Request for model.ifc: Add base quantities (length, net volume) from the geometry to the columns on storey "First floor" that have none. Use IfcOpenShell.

First a look at what the model holds.

```python
import ifcopenshell
import ifcopenshell.util.element
import ifcopenshell.util.unit

model = ifcopenshell.open("model.ifc")
print(model.schema)
for unit_type in ("LENGTHUNIT", "AREAUNIT", "VOLUMEUNIT"):
    print(unit_type, ifcopenshell.util.unit.calculate_unit_scale(model, unit_type))
storey = next(s for s in model.by_type("IfcBuildingStorey") if s.Name == "First floor")
columns = [e for e in ifcopenshell.util.element.get_decomposition(storey) if e.is_a("IfcColumn")]
for e in sorted(columns, key=lambda e: e.id()):
    print(e.id(), e.is_a(), e.Name, list(ifcopenshell.util.element.get_psets(e, qtos_only=True)), sep=" | ")
```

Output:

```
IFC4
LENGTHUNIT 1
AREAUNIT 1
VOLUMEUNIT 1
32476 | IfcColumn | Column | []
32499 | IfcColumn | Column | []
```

```python
import ifcopenshell
import ifcopenshell.api.pset
import ifcopenshell.geom
import ifcopenshell.util.element
import ifcopenshell.util.shape
import ifcopenshell.util.unit

model = ifcopenshell.open("model.ifc")
unit_scale = ifcopenshell.util.unit.calculate_unit_scale(model)
volume_scale = ifcopenshell.util.unit.calculate_unit_scale(model, "VOLUMEUNIT")
settings = ifcopenshell.geom.settings()

storey = next(s for s in model.by_type("IfcBuildingStorey") if s.Name == "First floor")
columns = [e for e in ifcopenshell.util.element.get_decomposition(storey) if e.is_a("IfcColumn")]

for e in sorted(columns, key=lambda e: e.id()):
    if ifcopenshell.util.element.get_psets(e, qtos_only=True, should_inherit=False):
        continue
    # Geometry comes back in metres, in the element's own axes.
    shape = ifcopenshell.geom.create_shape(settings, e)
    values = {
        "Length": ifcopenshell.util.shape.get_z(shape.geometry) / unit_scale,
        "NetVolume": ifcopenshell.util.shape.get_volume(shape.geometry) / volume_scale,
    }
    qto = ifcopenshell.api.pset.add_qto(model, product=e, name="Qto_ColumnBaseQuantities")
    ifcopenshell.api.pset.edit_qto(model, qto=qto, properties=values)
    print(e.id(), {k: round(v, 3) for k, v in values.items()})

model.write("model_rev.ifc")
```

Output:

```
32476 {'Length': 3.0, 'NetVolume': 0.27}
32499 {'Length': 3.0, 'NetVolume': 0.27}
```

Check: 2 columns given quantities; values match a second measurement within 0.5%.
